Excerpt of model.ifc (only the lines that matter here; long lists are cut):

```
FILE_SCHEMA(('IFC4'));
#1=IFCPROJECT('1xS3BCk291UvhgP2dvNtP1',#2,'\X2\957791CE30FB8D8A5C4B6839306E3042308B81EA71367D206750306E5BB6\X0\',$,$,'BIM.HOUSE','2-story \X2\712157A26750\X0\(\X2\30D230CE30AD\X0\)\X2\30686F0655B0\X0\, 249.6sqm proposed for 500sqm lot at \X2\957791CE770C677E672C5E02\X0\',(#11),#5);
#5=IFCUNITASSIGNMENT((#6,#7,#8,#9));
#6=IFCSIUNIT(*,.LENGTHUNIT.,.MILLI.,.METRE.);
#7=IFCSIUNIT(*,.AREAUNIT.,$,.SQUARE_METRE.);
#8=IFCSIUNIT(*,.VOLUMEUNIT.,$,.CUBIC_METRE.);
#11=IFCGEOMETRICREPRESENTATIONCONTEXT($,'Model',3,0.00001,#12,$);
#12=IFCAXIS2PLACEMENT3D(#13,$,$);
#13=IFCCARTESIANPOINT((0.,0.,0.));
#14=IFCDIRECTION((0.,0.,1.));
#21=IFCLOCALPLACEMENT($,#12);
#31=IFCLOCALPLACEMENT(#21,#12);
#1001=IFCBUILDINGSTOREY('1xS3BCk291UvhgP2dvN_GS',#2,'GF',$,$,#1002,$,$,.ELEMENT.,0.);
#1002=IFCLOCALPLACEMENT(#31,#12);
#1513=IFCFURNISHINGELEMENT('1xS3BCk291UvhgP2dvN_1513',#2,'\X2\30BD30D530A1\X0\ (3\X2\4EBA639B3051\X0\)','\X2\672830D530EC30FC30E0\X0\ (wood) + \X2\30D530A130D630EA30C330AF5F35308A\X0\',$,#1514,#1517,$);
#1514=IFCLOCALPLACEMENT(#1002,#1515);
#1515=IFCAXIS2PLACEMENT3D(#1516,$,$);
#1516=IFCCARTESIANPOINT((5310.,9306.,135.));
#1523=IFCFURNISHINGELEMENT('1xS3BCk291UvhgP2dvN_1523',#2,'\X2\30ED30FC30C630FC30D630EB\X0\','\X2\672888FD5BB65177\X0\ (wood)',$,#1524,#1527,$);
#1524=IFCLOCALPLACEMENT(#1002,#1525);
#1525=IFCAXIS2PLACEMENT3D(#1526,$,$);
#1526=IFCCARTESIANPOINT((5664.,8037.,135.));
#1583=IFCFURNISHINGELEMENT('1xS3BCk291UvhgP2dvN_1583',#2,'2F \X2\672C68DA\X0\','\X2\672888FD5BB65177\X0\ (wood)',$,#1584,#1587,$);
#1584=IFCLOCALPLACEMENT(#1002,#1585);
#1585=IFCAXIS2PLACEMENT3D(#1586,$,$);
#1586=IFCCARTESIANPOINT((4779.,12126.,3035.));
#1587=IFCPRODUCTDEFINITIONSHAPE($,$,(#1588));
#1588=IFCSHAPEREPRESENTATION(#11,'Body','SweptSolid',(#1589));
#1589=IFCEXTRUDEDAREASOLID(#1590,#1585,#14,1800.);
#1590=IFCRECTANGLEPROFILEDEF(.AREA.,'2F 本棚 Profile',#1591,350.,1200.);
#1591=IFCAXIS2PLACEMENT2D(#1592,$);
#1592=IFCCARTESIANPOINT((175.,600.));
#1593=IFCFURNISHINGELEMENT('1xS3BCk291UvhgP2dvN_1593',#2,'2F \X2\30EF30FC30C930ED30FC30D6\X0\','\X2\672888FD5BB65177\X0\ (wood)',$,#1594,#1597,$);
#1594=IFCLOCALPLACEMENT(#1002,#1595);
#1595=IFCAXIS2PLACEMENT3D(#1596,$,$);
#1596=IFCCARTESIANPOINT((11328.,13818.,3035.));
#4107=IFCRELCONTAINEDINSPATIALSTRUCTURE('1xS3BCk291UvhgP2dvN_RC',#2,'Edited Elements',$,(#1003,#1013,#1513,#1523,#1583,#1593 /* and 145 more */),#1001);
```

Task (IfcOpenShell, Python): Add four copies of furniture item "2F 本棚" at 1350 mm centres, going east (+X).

```python
import numpy as np
import ifcopenshell
import ifcopenshell.api.geometry
import ifcopenshell.api.root
import ifcopenshell.util.element
import ifcopenshell.util.placement
import ifcopenshell.util.unit

model = ifcopenshell.open("model.ifc")
unit_scale = ifcopenshell.util.unit.calculate_unit_scale(model)


def reuse_history(source, copy):
    """copy_class also copies each property set's owner history, people and application; keep the originals."""
    for rel in copy.IsDefinedBy:
        if rel.is_a("IfcRelDefinesByProperties") and (history := rel.RelatingPropertyDefinition.OwnerHistory):
            rel.RelatingPropertyDefinition.OwnerHistory = source.OwnerHistory
            ifcopenshell.util.element.remove_deep2(model, history)


source = model.by_guid("1xS3BCk291UvhgP2dvN_1583")
base = ifcopenshell.util.placement.get_local_placement(source.ObjectPlacement)
step = np.array([1.0, 0.0, 0.0]) * 1.35 / unit_scale

for i in range(1, 5):
    copy = ifcopenshell.api.root.copy_class(model, product=source)
    copy.Representation = ifcopenshell.util.element.copy_deep(
        model, source.Representation, exclude=["IfcGeometricRepresentationContext", "IfcRepresentationMap"]
    )
    reuse_history(source, copy)
    matrix = base.copy()
    matrix[:3, 3] += i * step
    print("added at", matrix[:3, 3].round(3) + 0.0)
    ifcopenshell.api.geometry.edit_object_placement(model, product=copy, matrix=matrix, is_si=False)

model.write("model-out.ifc")
```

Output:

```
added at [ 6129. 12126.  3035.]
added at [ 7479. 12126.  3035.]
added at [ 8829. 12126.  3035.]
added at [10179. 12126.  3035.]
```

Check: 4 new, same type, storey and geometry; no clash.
